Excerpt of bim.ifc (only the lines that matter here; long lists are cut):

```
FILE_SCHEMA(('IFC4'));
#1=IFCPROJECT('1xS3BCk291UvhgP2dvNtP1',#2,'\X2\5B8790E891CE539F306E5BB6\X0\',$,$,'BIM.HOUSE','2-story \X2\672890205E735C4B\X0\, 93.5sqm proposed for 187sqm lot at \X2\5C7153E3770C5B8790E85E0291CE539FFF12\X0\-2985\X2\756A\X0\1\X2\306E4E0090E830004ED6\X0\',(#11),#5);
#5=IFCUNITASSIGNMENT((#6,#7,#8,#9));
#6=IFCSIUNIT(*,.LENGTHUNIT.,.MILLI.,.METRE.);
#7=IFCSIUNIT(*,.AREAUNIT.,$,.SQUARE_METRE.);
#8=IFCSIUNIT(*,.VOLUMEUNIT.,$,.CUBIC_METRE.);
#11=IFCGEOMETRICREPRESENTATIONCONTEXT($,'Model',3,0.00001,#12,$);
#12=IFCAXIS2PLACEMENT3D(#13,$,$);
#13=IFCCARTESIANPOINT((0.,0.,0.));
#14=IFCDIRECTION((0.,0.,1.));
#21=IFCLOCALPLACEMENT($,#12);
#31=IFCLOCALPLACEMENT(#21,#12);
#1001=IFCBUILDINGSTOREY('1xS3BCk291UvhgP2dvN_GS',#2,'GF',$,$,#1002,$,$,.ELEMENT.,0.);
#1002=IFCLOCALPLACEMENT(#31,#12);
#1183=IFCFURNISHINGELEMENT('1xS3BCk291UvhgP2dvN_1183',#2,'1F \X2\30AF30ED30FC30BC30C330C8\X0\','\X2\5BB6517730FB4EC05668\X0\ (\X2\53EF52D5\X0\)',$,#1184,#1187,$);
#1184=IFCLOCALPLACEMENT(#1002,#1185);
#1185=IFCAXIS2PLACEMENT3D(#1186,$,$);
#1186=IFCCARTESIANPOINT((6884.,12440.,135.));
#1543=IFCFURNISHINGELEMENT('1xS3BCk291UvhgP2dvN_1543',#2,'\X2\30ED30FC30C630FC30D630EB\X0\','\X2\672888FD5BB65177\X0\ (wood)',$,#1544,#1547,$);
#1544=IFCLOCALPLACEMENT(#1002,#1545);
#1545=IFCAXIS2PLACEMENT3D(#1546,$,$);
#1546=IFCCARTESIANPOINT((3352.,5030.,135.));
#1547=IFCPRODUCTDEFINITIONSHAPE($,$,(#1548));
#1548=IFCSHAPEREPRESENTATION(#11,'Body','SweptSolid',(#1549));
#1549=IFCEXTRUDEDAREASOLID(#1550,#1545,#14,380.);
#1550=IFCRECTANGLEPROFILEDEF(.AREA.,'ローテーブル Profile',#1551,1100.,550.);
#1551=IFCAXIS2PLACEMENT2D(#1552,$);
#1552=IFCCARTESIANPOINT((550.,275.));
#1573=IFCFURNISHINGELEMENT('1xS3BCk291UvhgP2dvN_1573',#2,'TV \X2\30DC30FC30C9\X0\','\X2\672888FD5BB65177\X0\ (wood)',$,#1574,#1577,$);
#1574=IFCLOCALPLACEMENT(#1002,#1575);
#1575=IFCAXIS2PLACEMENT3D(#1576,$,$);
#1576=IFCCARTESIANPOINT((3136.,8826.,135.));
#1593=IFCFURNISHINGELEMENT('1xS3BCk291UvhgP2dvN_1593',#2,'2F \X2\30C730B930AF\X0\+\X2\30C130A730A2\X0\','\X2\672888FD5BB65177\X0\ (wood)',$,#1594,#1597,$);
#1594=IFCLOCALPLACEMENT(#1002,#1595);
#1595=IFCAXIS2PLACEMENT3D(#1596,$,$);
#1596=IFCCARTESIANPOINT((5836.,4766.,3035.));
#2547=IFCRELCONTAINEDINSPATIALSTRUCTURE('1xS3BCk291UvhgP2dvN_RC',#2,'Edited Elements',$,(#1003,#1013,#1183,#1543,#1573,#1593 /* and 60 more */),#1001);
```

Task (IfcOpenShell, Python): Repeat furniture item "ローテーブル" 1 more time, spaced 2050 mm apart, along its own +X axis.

```python
import ifcopenshell
import ifcopenshell.api.geometry
import ifcopenshell.api.root
import ifcopenshell.util.element
import ifcopenshell.util.placement

model = ifcopenshell.open("bim.ifc")


def reuse_history(source, copy):
    """copy_class also copies each property set's owner history, people and application; keep the originals."""
    for rel in copy.IsDefinedBy:
        if rel.is_a("IfcRelDefinesByProperties") and (history := rel.RelatingPropertyDefinition.OwnerHistory):
            rel.RelatingPropertyDefinition.OwnerHistory = source.OwnerHistory
            ifcopenshell.util.element.remove_deep2(model, history)


source = model.by_guid("1xS3BCk291UvhgP2dvN_1543")
base = ifcopenshell.util.placement.get_local_placement(source.ObjectPlacement)
step = base[:3, 0] * 2050.0

for i in range(1, 2):
    copy = ifcopenshell.api.root.copy_class(model, product=source)
    copy.Representation = ifcopenshell.util.element.copy_deep(
        model, source.Representation, exclude=["IfcGeometricRepresentationContext", "IfcRepresentationMap"]
    )
    reuse_history(source, copy)
    matrix = base.copy()
    matrix[:3, 3] += i * step
    print("added at", matrix[:3, 3].round(3) + 0.0)
    ifcopenshell.api.geometry.edit_object_placement(model, product=copy, matrix=matrix, is_si=False)

model.write("bim_v2.ifc")
```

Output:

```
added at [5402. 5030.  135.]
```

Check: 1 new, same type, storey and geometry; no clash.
